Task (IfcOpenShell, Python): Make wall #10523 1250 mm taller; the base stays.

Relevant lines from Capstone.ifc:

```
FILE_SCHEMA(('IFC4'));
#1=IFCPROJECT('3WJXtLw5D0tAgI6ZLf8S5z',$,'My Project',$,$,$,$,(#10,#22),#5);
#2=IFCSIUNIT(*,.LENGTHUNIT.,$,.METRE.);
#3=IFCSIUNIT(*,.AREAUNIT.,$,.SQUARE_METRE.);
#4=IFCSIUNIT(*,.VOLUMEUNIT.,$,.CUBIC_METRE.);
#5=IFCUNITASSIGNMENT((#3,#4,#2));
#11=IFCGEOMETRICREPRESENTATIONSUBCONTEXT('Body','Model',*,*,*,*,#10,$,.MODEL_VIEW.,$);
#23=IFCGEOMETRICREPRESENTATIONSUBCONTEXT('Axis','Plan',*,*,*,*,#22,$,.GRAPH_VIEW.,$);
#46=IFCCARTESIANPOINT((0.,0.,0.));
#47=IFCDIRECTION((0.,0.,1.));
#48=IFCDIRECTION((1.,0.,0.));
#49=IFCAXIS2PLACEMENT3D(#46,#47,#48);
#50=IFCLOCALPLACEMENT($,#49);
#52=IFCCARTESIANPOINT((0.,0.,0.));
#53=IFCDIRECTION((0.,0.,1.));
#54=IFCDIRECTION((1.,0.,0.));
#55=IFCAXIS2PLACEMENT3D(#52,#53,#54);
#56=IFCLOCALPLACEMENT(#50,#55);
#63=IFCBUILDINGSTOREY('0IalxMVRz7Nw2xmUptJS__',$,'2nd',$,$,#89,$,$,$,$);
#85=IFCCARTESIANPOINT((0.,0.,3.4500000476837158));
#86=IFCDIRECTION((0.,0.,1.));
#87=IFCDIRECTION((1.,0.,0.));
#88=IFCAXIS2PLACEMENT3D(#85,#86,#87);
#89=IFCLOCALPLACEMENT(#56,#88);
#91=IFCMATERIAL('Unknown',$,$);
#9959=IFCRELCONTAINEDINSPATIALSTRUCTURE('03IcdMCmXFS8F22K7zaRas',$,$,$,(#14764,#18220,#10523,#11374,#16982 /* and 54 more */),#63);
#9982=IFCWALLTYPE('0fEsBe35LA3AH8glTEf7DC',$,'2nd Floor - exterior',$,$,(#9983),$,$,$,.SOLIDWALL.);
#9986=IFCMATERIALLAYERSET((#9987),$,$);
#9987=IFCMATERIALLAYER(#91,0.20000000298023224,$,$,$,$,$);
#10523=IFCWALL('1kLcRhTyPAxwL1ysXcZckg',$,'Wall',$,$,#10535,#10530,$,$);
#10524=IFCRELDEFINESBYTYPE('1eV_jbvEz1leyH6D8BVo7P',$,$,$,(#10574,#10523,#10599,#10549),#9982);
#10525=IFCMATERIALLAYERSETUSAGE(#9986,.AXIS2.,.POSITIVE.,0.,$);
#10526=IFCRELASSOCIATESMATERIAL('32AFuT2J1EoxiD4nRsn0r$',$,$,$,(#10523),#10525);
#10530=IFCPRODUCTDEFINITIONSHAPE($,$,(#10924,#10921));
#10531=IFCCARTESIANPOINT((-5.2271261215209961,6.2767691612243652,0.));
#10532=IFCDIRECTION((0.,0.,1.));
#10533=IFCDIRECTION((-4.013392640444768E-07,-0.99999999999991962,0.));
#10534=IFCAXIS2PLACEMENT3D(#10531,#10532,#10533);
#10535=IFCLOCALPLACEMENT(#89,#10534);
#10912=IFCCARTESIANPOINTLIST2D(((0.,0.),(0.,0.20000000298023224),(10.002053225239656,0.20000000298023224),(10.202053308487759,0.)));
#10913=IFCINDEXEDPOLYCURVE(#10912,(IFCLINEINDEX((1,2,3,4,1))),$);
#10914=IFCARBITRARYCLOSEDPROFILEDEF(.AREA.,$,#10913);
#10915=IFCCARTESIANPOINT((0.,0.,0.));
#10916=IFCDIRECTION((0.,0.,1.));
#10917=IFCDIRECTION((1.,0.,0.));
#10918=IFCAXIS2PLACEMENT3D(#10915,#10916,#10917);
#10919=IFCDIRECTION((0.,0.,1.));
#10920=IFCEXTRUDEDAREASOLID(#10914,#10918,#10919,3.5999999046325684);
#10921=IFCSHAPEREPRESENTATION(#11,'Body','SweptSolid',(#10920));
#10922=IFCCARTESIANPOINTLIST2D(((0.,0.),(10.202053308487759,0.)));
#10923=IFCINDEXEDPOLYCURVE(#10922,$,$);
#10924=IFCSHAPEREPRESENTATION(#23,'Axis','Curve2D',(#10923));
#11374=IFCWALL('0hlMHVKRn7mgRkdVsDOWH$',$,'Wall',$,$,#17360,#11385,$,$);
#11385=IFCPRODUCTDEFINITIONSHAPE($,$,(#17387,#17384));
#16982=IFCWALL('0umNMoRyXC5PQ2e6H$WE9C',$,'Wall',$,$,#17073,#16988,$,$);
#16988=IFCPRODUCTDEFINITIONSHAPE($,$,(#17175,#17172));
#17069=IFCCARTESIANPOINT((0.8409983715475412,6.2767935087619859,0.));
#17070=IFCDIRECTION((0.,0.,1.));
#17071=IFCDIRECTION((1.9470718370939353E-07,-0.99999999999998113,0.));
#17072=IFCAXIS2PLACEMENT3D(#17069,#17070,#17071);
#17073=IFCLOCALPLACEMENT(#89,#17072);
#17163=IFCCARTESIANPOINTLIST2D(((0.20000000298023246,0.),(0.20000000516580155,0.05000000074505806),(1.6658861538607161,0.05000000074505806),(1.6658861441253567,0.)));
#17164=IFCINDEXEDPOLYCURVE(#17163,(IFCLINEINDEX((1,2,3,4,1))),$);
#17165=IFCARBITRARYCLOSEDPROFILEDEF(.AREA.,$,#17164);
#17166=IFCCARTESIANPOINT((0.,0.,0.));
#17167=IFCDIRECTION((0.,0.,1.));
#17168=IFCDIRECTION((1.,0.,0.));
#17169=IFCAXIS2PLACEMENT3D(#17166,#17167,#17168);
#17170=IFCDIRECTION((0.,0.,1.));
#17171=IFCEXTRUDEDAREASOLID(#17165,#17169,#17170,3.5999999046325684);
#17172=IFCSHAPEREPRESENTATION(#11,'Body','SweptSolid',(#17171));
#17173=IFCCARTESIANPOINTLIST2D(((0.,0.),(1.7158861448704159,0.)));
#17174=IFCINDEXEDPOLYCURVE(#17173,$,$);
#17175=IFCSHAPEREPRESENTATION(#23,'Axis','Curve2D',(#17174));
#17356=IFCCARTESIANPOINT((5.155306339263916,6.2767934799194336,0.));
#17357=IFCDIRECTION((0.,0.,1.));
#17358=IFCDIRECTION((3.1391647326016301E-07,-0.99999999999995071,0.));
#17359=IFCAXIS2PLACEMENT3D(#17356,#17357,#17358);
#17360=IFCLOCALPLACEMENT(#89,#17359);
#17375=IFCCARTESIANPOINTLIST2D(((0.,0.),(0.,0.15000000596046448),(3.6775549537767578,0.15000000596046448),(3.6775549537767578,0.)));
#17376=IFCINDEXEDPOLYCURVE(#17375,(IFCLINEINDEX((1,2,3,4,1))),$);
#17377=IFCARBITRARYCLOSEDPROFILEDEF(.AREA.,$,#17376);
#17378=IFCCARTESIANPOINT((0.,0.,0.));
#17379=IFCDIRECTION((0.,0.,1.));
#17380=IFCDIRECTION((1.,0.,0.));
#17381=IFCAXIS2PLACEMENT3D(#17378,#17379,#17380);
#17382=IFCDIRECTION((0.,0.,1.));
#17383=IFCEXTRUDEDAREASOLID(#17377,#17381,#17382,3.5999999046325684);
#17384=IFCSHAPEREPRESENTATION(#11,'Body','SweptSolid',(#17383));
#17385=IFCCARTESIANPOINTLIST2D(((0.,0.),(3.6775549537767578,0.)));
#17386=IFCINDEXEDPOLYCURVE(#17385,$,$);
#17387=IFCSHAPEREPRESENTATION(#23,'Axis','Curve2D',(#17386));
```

```python
import ifcopenshell
import ifcopenshell.geom
import ifcopenshell.util.representation
import ifcopenshell.util.shape
import ifcopenshell.util.unit

model = ifcopenshell.open("Capstone.ifc")
unit_scale = ifcopenshell.util.unit.calculate_unit_scale(model)
settings = ifcopenshell.geom.settings()


def volume(element):
    """Net volume in cubic metres, openings subtracted."""
    shape = ifcopenshell.geom.create_shape(settings, element)
    return ifcopenshell.util.shape.get_volume(shape.geometry)


wall = model.by_id(10523)
before = volume(wall)

body = ifcopenshell.util.representation.get_representation(wall, "Model", "Body")
solid = body.Items[0]
old_height = solid.Depth
solid.Depth += 1.25 / unit_scale
after = volume(wall)

print(f"height {old_height:g} -> {solid.Depth:g}, volume {before:.3f} -> {after:.3f} m3")

model.write("Capstone_edited.ifc")
```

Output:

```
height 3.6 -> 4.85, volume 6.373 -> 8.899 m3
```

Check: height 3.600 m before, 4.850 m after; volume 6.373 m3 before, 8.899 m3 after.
